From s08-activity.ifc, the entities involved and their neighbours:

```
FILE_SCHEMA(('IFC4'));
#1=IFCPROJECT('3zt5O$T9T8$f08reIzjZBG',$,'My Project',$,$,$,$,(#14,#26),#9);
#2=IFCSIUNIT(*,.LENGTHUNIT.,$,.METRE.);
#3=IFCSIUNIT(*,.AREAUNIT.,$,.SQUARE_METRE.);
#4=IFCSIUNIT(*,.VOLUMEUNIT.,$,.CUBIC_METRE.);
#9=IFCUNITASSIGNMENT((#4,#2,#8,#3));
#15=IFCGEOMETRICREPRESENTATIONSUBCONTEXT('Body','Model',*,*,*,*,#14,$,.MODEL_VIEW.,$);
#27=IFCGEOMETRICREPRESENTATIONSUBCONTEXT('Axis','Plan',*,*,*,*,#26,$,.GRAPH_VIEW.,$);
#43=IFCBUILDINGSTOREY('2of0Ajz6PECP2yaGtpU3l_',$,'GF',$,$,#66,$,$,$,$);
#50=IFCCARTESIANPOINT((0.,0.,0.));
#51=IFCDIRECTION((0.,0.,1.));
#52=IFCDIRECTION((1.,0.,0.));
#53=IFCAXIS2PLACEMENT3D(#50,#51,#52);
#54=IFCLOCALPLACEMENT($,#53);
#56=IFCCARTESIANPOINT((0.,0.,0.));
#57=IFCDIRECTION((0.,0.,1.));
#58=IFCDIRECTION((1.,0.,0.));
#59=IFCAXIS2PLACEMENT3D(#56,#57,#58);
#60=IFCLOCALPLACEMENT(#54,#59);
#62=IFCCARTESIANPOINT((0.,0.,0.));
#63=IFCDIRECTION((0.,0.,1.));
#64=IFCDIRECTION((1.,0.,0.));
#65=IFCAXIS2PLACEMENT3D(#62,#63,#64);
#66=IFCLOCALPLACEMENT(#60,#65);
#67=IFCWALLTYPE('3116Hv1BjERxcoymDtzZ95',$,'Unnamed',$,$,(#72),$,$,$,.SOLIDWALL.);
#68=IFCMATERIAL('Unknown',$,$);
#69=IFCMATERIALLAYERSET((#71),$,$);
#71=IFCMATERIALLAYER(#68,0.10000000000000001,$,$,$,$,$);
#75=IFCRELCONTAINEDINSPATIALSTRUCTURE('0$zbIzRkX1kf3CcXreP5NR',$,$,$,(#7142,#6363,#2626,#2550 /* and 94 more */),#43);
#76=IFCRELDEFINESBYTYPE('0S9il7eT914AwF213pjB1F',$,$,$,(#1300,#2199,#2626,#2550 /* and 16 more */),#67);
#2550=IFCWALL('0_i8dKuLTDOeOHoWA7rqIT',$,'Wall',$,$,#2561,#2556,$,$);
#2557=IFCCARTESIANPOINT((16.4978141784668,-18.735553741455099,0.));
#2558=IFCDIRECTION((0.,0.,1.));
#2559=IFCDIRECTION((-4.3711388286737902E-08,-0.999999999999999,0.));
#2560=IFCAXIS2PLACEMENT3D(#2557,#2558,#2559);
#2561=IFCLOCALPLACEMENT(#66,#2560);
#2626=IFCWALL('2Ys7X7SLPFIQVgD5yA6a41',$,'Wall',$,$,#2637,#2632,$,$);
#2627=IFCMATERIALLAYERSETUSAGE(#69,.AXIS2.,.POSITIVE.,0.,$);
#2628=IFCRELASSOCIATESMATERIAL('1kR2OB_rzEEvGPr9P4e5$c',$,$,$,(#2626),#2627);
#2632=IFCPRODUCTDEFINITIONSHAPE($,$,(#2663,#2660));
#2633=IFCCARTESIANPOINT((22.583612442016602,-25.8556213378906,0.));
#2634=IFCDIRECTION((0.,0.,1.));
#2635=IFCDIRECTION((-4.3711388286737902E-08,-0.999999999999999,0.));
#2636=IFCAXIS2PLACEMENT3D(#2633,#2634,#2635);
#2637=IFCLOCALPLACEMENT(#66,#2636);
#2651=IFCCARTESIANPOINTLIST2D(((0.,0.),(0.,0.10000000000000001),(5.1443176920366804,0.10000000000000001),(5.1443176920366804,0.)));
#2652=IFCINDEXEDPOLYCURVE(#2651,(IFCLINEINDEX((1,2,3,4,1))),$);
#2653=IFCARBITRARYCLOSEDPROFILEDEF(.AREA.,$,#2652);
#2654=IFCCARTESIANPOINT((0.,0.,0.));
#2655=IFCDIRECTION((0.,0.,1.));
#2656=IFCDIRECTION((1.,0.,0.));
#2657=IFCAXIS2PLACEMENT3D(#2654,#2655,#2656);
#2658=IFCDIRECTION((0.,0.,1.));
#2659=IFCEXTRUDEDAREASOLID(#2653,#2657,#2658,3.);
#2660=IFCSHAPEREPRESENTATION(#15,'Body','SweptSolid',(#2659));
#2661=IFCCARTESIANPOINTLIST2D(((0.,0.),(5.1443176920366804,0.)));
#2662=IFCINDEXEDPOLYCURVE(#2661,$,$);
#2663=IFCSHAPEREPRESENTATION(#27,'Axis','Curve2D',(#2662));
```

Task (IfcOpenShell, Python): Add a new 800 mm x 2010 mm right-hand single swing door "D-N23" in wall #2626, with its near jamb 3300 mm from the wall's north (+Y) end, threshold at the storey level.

```python
import numpy as np
import ifcopenshell
import ifcopenshell.api.feature
import ifcopenshell.api.geometry
import ifcopenshell.api.root
import ifcopenshell.api.spatial
import ifcopenshell.geom
import ifcopenshell.util.element
import ifcopenshell.util.placement
import ifcopenshell.util.representation
import ifcopenshell.util.shape
import ifcopenshell.util.unit

model = ifcopenshell.open("s08-activity.ifc")
unit_scale = ifcopenshell.util.unit.calculate_unit_scale(model)
settings = ifcopenshell.geom.settings()


def volume(element):
    """Net volume in cubic metres, openings subtracted."""
    shape = ifcopenshell.geom.create_shape(settings, element)
    return ifcopenshell.util.shape.get_volume(shape.geometry)


wall = model.by_guid("2Ys7X7SLPFIQVgD5yA6a41")
storey = ifcopenshell.util.element.get_container(wall, ifc_class="IfcBuildingStorey")
context = ifcopenshell.util.representation.get_context(model, "Model", "Body", "MODEL_VIEW")
before = volume(wall)

width, height, from_end, sill = 0.8, 2.01, 3.3, 0.0  # metres

# The wall runs along its own X axis, and the end named is its -X end.
wall_shape = ifcopenshell.geom.create_shape(settings, wall)
x, y, z = ifcopenshell.util.shape.get_vertices(wall_shape.geometry).T
start = x.min() + from_end
face, thickness = float(y.min()), float(y.max() - y.min())
wall_matrix = ifcopenshell.util.placement.get_local_placement(wall.ObjectPlacement)
level = ifcopenshell.util.placement.get_local_placement(storey.ObjectPlacement)[2, 3]


def in_wall(x, y):
    """Placement at x, y metres in the wall's axes, at sill height."""
    matrix = wall_matrix.copy()
    matrix[:, 3] = wall_matrix @ np.array([x / unit_scale, y / unit_scale, 0.0, 1.0])
    matrix[2, 3] = level + sill / unit_scale
    return matrix


# Opening: a box that overshoots both wall faces by 50 mm.
opening = ifcopenshell.api.root.create_entity(model, ifc_class="IfcOpeningElement", predefined_type="OPENING")
box = ifcopenshell.api.geometry.add_wall_representation(
    model, context=context, length=width, height=height, thickness=thickness + 0.1
)
ifcopenshell.api.geometry.assign_representation(model, product=opening, representation=box)
ifcopenshell.api.geometry.edit_object_placement(model, product=opening, matrix=in_wall(start, face - 0.05), is_si=False)
ifcopenshell.api.feature.add_feature(model, feature=opening, element=wall)

door = ifcopenshell.api.root.create_entity(model, ifc_class="IfcDoor", name="D-N23", predefined_type="DOOR")
door.OverallWidth, door.OverallHeight = width / unit_scale, height / unit_scale
door.OperationType = "SINGLE_SWING_RIGHT"
body = ifcopenshell.api.geometry.add_door_representation(
    model,
    context=context,
    overall_width=door.OverallWidth,
    overall_height=door.OverallHeight,
    operation_type="SINGLE_SWING_RIGHT",
    lining_properties={"LiningDepth": thickness / unit_scale, "ThresholdDepth": thickness / unit_scale},
)
ifcopenshell.api.geometry.assign_representation(model, product=door, representation=body)
ifcopenshell.api.spatial.assign_container(model, products=[door], relating_structure=storey)
ifcopenshell.api.feature.add_filling(model, opening=opening, element=door)

# The lining spans the wall, so the door starts at the wall face.
ifcopenshell.api.geometry.edit_object_placement(model, product=door, matrix=in_wall(start, face), is_si=False)

after = volume(wall)

print(f"wall volume {before:.3f} -> {after:.3f} m3")

model.write("s08-activity_updated.ifc")
```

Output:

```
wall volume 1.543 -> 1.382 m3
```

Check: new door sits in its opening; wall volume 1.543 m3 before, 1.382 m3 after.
